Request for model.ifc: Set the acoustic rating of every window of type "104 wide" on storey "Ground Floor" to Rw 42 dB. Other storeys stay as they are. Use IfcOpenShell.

First a look at what the model holds.

```python
import ifcopenshell
import ifcopenshell.util.element

model = ifcopenshell.open("model.ifc")
print(model.schema)
storey = next(s for s in model.by_type("IfcBuildingStorey") if s.Name == "Ground Floor")
windows = [e for e in ifcopenshell.util.element.get_decomposition(storey) if e.is_a("IfcWindow")]
seen = {}
for e in windows:
    element_type = ifcopenshell.util.element.get_type(e)
    key = (element_type.Name if element_type != e and element_type else None, ifcopenshell.util.element.get_pset(e, "Pset_WindowCommon", "AcousticRating"))
    seen[key] = seen.get(key, 0) + 1
for (name, value), count in sorted(seen.items(), key=str):
    print(count, "x", name, "|", value)
```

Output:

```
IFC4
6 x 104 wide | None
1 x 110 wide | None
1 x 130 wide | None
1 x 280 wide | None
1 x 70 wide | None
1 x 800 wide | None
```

```python
import ifcopenshell
import ifcopenshell.api.pset
import ifcopenshell.util.element

model = ifcopenshell.open("model.ifc")

storey = next(s for s in model.by_type("IfcBuildingStorey") if s.Name == "Ground Floor")
windows = [e for e in ifcopenshell.util.element.get_decomposition(storey) if e.is_a("IfcWindow")]

count = 0
for e in windows:
    element_type = ifcopenshell.util.element.get_type(e)
    if element_type in (None, e) or element_type.Name != "104 wide":
        continue
    # add_pset returns the element's existing set when there is one.
    pset = ifcopenshell.api.pset.add_pset(model, product=e, name="Pset_WindowCommon")
    ifcopenshell.api.pset.edit_pset(model, pset=pset, properties={"AcousticRating": "Rw 42 dB"})
    count += 1

print(count, "windows updated")

model.write("model_updated.ifc")
```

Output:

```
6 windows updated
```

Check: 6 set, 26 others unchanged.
